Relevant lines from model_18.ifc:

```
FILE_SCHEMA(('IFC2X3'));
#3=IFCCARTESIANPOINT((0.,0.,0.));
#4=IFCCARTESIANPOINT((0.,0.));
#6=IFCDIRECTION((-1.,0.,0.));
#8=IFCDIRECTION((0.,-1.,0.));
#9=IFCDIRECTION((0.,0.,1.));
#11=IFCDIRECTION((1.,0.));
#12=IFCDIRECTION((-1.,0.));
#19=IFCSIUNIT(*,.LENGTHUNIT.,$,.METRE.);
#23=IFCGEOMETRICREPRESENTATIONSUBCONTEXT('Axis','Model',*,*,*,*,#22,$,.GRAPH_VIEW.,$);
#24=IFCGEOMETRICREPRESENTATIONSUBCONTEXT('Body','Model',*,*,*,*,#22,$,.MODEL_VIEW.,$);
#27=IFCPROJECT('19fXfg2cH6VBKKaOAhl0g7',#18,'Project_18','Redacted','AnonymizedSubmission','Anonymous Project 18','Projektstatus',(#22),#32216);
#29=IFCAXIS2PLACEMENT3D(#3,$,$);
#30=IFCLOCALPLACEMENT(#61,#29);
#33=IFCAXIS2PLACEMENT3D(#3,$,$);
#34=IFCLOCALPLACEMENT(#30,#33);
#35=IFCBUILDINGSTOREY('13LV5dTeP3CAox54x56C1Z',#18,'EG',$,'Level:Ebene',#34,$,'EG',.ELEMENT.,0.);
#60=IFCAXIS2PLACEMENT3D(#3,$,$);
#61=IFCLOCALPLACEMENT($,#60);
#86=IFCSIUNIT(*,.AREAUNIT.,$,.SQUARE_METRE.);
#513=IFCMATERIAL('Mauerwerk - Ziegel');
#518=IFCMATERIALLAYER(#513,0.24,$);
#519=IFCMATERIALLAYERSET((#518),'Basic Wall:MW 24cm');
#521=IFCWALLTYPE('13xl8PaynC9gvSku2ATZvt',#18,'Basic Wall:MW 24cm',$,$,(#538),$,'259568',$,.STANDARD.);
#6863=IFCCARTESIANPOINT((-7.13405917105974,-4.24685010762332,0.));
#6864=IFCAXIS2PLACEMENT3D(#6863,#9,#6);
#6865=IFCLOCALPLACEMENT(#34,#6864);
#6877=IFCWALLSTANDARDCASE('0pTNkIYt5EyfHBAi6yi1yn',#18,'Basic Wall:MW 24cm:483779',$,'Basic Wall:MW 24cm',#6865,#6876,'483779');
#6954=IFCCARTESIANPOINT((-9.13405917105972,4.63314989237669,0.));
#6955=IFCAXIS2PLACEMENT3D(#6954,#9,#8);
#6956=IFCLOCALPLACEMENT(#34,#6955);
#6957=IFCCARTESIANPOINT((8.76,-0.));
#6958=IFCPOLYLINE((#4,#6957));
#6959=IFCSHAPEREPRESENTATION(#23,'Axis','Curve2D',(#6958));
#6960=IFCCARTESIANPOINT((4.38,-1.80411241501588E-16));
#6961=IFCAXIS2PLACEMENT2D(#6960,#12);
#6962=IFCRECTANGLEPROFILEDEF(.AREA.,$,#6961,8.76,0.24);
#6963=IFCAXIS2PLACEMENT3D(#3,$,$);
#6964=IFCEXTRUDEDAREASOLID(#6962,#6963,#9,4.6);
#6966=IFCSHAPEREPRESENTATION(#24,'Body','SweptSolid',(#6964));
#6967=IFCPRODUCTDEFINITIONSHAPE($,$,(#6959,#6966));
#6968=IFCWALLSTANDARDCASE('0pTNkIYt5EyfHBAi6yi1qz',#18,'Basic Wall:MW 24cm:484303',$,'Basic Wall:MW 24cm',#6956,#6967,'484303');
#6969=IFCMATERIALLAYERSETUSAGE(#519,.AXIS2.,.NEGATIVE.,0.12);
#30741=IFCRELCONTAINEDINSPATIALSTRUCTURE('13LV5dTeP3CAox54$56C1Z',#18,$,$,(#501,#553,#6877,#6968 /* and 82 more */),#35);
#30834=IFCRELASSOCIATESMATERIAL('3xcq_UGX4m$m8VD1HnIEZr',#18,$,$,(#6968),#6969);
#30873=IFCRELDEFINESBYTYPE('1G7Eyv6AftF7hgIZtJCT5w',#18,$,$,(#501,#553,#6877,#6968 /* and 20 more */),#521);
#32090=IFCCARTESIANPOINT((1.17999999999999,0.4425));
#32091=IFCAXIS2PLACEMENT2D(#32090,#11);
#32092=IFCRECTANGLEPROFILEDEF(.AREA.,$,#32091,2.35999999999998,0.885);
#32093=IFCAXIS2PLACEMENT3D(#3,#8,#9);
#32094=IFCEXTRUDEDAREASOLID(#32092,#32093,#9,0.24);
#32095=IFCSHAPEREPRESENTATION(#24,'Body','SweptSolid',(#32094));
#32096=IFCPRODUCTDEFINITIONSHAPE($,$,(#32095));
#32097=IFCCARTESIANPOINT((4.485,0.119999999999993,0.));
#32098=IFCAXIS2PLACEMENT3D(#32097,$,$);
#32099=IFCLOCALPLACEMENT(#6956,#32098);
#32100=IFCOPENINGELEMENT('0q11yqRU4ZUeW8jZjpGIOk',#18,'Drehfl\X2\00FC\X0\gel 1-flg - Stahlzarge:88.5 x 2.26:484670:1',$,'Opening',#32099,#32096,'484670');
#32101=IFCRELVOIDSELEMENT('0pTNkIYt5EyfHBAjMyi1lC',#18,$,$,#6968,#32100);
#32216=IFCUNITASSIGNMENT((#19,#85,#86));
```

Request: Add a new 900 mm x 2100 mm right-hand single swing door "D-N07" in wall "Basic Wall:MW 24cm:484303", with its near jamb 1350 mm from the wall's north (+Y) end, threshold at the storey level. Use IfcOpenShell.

```python
import numpy as np
import ifcopenshell
import ifcopenshell.api.feature
import ifcopenshell.api.geometry
import ifcopenshell.api.root
import ifcopenshell.api.spatial
import ifcopenshell.api.type
import ifcopenshell.geom
import ifcopenshell.util.element
import ifcopenshell.util.placement
import ifcopenshell.util.representation
import ifcopenshell.util.shape
import ifcopenshell.util.unit

model = ifcopenshell.open("model_18.ifc")
unit_scale = ifcopenshell.util.unit.calculate_unit_scale(model)
settings = ifcopenshell.geom.settings()


def volume(element):
    """Net volume in cubic metres, openings subtracted."""
    shape = ifcopenshell.geom.create_shape(settings, element)
    return ifcopenshell.util.shape.get_volume(shape.geometry)


wall = model.by_id(6968)
storey = ifcopenshell.util.element.get_container(wall, ifc_class="IfcBuildingStorey")
context = ifcopenshell.util.representation.get_context(model, "Model", "Body", "MODEL_VIEW")
before = volume(wall)

width, height, from_end, sill = 0.9, 2.1, 1.35, 0.0  # metres

# The wall runs along its own X axis, and the end named is its -X end.
wall_shape = ifcopenshell.geom.create_shape(settings, wall)
x, y, z = ifcopenshell.util.shape.get_vertices(wall_shape.geometry).T
start = x.min() + from_end
face, thickness = float(y.min()), float(y.max() - y.min())
wall_matrix = ifcopenshell.util.placement.get_local_placement(wall.ObjectPlacement)
level = ifcopenshell.util.placement.get_local_placement(storey.ObjectPlacement)[2, 3]


def in_wall(x, y):
    """Placement at x, y metres in the wall's axes, at sill height."""
    matrix = wall_matrix.copy()
    matrix[:, 3] = wall_matrix @ np.array([x / unit_scale, y / unit_scale, 0.0, 1.0])
    matrix[2, 3] = level + sill / unit_scale
    return matrix


# Opening: a box that overshoots both wall faces by 50 mm.
opening = ifcopenshell.api.root.create_entity(model, ifc_class="IfcOpeningElement")
box = ifcopenshell.api.geometry.add_wall_representation(
    model, context=context, length=width, height=height, thickness=thickness + 0.1
)
ifcopenshell.api.geometry.assign_representation(model, product=opening, representation=box)
ifcopenshell.api.geometry.edit_object_placement(model, product=opening, matrix=in_wall(start, face - 0.05), is_si=False)
ifcopenshell.api.feature.add_feature(model, feature=opening, element=wall)

door = ifcopenshell.api.root.create_entity(model, ifc_class="IfcDoor", name="D-N07")
door.OverallWidth, door.OverallHeight = width / unit_scale, height / unit_scale
body = ifcopenshell.api.geometry.add_door_representation(
    model,
    context=context,
    overall_width=door.OverallWidth,
    overall_height=door.OverallHeight,
    operation_type="SINGLE_SWING_RIGHT",
    lining_properties={"LiningDepth": thickness / unit_scale, "ThresholdDepth": thickness / unit_scale},
)
ifcopenshell.api.geometry.assign_representation(model, product=door, representation=body)
ifcopenshell.api.spatial.assign_container(model, products=[door], relating_structure=storey)
fills = ifcopenshell.api.feature.add_filling(model, opening=opening, element=door)
fills.OwnerHistory = door.OwnerHistory  # required in IFC2X3

# IFC2X3 keeps the operation on the door style.
style = ifcopenshell.api.root.create_entity(model, ifc_class="IfcDoorStyle", name="D-N07")
style.OperationType, style.ConstructionType = "SINGLE_SWING_RIGHT", "NOTDEFINED"
style.ParameterTakesPrecedence = style.Sizeable = False
ifcopenshell.api.type.assign_type(model, related_objects=[door], relating_type=style)

# The lining spans the wall, so the door starts at the wall face.
ifcopenshell.api.geometry.edit_object_placement(model, product=door, matrix=in_wall(start, face), is_si=False)

after = volume(wall)

print(f"wall volume {before:.3f} -> {after:.3f} m3")

model.write("model_18_rev.ifc")
```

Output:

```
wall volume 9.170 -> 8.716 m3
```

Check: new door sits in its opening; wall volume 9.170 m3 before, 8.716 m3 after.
